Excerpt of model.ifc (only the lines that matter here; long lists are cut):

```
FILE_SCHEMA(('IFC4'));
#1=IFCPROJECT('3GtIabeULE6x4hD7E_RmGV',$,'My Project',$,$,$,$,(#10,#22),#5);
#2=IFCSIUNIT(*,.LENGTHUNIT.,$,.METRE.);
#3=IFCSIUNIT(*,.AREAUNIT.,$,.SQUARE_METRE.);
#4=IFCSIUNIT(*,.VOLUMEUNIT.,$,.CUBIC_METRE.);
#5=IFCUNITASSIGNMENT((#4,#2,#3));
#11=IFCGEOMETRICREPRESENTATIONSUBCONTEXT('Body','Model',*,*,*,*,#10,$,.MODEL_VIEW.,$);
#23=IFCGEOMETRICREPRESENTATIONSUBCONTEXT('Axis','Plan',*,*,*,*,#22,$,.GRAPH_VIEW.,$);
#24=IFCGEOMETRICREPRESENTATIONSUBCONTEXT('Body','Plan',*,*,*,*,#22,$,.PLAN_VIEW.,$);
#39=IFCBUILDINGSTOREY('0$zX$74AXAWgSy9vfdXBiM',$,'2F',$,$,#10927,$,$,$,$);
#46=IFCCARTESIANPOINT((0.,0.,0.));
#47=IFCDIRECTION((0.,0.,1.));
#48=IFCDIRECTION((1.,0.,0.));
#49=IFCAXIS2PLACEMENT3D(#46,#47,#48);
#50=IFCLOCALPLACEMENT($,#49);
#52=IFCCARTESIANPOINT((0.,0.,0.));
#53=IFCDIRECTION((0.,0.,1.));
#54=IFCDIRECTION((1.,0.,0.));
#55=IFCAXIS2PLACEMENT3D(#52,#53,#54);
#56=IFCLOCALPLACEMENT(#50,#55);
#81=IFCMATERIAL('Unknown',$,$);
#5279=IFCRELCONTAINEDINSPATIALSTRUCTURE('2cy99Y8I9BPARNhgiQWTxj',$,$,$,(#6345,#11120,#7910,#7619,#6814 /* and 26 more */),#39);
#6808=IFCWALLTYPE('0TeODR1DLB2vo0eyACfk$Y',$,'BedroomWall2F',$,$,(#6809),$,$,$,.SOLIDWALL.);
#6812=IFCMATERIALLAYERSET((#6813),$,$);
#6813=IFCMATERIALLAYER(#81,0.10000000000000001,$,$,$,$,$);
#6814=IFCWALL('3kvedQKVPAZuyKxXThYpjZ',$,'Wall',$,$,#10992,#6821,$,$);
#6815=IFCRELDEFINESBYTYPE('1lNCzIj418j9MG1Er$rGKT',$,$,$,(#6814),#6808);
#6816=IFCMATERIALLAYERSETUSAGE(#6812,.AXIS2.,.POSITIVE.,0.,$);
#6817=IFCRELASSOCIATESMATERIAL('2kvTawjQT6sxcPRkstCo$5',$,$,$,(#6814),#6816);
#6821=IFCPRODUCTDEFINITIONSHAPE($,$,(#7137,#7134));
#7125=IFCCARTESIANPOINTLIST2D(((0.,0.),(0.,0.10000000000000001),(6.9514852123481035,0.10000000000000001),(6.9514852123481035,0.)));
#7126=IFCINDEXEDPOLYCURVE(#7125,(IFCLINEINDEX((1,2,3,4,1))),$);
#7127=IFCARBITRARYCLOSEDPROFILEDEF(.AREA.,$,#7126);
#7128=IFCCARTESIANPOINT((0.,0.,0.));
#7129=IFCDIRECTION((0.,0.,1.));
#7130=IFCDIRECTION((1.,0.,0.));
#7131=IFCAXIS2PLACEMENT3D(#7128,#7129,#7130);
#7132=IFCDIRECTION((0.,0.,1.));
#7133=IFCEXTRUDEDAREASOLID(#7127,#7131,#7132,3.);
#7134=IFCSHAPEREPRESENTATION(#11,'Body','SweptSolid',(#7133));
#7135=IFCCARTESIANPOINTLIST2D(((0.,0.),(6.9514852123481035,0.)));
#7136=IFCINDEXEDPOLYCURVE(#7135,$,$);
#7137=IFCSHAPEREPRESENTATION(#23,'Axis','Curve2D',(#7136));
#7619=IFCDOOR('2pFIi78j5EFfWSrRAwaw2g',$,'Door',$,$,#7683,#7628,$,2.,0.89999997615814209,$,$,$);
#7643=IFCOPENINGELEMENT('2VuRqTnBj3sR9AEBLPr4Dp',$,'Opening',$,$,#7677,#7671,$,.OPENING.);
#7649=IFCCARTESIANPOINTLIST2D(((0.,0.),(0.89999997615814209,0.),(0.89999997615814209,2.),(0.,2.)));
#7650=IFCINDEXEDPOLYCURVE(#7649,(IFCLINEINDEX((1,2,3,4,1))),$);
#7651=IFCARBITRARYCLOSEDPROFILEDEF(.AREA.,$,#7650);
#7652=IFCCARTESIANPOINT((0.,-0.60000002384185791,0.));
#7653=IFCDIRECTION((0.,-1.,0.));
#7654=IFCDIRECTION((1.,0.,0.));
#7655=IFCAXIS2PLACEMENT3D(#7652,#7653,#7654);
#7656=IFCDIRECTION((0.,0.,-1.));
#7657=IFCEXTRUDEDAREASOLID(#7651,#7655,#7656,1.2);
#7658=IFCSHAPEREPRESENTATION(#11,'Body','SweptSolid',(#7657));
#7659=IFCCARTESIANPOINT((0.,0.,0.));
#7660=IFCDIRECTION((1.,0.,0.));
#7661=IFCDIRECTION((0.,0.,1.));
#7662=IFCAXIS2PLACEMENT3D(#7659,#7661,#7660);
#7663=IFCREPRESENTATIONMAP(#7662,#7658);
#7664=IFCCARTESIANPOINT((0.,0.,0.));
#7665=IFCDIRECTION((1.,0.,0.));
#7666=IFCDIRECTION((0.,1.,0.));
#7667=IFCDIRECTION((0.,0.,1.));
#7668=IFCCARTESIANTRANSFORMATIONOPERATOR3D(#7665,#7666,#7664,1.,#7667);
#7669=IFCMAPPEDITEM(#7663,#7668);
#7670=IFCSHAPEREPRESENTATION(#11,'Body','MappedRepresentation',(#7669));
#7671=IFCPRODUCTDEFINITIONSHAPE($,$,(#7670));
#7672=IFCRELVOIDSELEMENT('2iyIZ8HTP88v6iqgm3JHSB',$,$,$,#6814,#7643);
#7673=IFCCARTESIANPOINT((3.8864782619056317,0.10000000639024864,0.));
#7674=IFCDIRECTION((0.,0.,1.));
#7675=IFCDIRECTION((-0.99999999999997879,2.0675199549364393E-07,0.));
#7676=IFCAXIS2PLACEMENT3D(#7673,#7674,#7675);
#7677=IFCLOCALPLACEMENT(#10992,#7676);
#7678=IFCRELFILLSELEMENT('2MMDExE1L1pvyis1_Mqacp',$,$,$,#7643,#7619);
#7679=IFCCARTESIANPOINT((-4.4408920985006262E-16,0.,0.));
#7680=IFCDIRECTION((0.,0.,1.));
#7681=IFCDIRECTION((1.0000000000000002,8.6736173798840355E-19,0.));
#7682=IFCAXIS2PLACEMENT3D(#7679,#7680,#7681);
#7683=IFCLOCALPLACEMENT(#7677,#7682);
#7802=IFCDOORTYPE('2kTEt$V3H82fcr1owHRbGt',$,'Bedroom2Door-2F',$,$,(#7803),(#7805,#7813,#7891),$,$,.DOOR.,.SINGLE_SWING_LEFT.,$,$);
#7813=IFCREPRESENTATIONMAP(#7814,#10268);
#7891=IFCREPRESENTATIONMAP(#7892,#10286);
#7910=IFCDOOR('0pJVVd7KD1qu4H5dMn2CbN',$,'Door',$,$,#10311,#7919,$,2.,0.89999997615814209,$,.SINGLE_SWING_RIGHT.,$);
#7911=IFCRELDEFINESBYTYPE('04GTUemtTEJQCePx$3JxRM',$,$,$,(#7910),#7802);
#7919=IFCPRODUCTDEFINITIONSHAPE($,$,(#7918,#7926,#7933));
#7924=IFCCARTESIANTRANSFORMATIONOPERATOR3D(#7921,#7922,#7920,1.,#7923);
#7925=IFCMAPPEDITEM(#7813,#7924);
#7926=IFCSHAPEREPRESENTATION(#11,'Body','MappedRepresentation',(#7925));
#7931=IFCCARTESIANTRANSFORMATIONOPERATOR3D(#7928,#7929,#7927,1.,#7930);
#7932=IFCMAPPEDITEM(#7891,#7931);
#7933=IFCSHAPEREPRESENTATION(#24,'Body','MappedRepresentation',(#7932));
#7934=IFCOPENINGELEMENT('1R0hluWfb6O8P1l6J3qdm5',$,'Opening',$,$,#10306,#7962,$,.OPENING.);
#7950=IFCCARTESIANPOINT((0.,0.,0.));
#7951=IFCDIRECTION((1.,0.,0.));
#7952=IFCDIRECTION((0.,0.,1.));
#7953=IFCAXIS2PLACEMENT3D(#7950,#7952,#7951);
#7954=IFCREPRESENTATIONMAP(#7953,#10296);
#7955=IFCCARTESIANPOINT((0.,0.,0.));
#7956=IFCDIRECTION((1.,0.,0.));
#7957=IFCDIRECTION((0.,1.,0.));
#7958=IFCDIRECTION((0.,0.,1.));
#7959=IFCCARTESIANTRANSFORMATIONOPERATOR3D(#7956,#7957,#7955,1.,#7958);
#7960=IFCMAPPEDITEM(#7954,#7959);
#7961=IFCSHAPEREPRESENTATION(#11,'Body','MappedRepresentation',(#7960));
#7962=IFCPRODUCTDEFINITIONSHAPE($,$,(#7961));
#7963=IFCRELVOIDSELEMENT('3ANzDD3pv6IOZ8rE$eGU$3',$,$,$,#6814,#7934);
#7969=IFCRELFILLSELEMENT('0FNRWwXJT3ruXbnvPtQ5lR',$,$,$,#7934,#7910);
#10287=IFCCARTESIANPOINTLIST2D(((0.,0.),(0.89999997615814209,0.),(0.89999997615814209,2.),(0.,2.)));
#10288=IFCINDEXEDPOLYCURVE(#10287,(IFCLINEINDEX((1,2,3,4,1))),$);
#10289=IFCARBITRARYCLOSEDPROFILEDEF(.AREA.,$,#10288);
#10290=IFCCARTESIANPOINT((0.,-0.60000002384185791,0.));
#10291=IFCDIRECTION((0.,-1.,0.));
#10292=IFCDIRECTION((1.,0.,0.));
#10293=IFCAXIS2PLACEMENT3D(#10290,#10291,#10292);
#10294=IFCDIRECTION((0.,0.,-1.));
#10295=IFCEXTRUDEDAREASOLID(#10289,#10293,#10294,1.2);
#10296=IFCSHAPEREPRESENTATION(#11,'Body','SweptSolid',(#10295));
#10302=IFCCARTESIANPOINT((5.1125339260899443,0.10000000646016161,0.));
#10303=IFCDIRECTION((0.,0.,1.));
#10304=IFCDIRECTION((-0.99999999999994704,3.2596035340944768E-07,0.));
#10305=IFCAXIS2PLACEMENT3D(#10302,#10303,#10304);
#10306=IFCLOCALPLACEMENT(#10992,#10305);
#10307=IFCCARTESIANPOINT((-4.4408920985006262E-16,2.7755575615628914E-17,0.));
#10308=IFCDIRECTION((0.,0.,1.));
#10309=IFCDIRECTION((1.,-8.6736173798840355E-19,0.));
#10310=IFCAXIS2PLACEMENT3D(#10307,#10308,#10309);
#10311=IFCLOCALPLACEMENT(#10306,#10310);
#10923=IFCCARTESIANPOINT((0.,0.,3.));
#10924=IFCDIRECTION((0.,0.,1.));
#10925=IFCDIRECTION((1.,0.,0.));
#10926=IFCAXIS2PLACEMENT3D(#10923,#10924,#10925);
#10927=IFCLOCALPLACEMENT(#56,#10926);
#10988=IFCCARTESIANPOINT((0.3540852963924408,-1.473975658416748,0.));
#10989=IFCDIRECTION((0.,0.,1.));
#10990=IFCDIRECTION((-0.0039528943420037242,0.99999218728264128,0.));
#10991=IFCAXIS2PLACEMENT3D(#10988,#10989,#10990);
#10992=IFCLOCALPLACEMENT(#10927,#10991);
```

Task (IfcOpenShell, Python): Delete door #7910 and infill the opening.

```python
import ifcopenshell
import ifcopenshell.api.feature
import ifcopenshell.api.root
import ifcopenshell.geom
import ifcopenshell.util.shape

model = ifcopenshell.open("model.ifc")
settings = ifcopenshell.geom.settings()


def volume(element):
    """Net volume in cubic metres, openings subtracted."""
    shape = ifcopenshell.geom.create_shape(settings, element)
    return ifcopenshell.util.shape.get_volume(shape.geometry)


door = model.by_guid("0pJVVd7KD1qu4H5dMn2CbN")
opening = door.FillsVoids[0].RelatingOpeningElement
wall = opening.VoidsElements[0].RelatingBuildingElement
before = volume(wall)

ifcopenshell.api.root.remove_product(model, product=door)
ifcopenshell.api.feature.remove_feature(model, feature=opening)

after = volume(wall)

print(f"wall volume {before:.3f} -> {after:.3f} m3")

model.write("model_updated.ifc")
```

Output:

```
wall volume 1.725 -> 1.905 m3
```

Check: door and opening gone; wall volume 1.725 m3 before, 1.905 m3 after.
